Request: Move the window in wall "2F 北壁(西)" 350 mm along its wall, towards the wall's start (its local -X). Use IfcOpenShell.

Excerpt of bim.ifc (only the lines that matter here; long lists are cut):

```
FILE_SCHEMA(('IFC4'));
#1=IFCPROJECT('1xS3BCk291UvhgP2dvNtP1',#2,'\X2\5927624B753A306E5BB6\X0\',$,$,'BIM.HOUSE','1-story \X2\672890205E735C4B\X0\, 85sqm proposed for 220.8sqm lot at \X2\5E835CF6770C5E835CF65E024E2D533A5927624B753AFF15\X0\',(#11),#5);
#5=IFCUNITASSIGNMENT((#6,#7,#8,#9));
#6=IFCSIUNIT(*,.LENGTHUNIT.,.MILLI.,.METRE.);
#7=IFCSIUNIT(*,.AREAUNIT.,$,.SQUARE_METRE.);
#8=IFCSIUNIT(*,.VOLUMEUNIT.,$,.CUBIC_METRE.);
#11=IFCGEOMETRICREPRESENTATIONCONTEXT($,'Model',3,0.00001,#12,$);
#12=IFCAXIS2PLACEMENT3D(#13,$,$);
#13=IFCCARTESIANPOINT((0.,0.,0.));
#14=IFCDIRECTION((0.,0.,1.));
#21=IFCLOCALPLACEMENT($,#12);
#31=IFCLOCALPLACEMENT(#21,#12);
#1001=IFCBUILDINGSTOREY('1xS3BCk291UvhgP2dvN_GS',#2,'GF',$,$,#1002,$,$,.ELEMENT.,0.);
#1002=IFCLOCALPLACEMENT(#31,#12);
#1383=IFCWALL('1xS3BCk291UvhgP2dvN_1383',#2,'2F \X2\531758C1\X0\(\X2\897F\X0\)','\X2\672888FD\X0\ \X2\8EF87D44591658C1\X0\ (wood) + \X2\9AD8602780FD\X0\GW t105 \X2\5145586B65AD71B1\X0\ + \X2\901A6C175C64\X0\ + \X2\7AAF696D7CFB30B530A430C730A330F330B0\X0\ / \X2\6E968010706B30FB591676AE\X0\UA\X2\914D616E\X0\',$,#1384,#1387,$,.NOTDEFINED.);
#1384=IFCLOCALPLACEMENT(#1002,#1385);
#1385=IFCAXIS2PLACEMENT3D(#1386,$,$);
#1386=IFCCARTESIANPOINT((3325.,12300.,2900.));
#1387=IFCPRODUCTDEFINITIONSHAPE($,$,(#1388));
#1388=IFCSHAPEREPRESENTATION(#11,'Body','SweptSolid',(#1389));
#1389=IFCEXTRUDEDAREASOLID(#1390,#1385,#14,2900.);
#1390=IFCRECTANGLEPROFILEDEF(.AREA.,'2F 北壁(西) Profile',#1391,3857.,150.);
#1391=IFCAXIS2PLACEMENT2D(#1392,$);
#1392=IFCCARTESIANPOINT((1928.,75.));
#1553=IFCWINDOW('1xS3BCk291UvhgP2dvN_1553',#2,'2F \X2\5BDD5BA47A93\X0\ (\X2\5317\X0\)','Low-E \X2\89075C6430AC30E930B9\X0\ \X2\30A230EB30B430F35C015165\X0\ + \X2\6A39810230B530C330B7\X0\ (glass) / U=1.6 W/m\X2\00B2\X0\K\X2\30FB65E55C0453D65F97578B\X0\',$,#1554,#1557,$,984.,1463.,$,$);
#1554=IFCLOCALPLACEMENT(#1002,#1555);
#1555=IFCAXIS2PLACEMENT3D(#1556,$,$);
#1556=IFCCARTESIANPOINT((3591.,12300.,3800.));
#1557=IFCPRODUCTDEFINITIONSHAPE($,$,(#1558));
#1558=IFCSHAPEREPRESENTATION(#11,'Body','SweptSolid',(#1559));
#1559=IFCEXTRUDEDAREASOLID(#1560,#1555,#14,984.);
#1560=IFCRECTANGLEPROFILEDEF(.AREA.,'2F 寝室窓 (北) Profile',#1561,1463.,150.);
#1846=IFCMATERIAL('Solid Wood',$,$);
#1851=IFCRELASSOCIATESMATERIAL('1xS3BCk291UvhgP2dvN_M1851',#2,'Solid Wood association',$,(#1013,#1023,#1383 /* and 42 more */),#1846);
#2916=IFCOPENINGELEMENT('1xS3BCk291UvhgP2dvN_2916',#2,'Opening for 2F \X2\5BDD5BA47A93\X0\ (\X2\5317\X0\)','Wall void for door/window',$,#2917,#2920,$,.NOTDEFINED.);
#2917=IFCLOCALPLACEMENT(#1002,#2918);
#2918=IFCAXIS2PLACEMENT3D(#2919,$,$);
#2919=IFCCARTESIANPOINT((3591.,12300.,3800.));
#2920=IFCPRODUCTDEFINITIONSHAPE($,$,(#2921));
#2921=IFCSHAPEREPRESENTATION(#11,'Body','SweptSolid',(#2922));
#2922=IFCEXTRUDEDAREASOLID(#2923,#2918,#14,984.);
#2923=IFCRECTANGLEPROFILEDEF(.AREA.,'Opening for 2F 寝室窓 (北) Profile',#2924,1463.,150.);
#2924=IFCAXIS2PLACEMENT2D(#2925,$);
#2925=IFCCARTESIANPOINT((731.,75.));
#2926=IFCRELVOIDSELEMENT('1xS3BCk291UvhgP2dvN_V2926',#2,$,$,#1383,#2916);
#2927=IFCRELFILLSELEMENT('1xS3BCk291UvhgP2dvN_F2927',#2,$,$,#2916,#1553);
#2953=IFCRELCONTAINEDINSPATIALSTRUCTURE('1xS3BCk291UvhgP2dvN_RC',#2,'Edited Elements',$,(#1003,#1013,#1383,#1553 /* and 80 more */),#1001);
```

```python
import ifcopenshell
import ifcopenshell.api.geometry
import ifcopenshell.util.placement
import ifcopenshell.util.unit

model = ifcopenshell.open("bim.ifc")
unit_scale = ifcopenshell.util.unit.calculate_unit_scale(model)

window = model.by_id(1553)
opening = window.FillsVoids[0].RelatingOpeningElement
wall = opening.VoidsElements[0].RelatingBuildingElement

wall_matrix = ifcopenshell.util.placement.get_local_placement(wall.ObjectPlacement)
shift = wall_matrix[:3, 0] * -0.35 / unit_scale
before = ifcopenshell.util.placement.get_local_placement(window.ObjectPlacement)[:3, 3].copy()

# The window is not placed relative to its opening, so move both.
for product in (opening, window):
    matrix = ifcopenshell.util.placement.get_local_placement(product.ObjectPlacement)
    matrix[:3, 3] += shift
    ifcopenshell.api.geometry.edit_object_placement(model, product=product, matrix=matrix, is_si=False)

after = ifcopenshell.util.placement.get_local_placement(window.ObjectPlacement)[:3, 3]
print("window moved by", (after - before).round(3) + 0.0)

model.write("bim_rev.ifc")
```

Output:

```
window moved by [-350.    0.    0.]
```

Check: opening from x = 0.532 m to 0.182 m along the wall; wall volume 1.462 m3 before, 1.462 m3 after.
